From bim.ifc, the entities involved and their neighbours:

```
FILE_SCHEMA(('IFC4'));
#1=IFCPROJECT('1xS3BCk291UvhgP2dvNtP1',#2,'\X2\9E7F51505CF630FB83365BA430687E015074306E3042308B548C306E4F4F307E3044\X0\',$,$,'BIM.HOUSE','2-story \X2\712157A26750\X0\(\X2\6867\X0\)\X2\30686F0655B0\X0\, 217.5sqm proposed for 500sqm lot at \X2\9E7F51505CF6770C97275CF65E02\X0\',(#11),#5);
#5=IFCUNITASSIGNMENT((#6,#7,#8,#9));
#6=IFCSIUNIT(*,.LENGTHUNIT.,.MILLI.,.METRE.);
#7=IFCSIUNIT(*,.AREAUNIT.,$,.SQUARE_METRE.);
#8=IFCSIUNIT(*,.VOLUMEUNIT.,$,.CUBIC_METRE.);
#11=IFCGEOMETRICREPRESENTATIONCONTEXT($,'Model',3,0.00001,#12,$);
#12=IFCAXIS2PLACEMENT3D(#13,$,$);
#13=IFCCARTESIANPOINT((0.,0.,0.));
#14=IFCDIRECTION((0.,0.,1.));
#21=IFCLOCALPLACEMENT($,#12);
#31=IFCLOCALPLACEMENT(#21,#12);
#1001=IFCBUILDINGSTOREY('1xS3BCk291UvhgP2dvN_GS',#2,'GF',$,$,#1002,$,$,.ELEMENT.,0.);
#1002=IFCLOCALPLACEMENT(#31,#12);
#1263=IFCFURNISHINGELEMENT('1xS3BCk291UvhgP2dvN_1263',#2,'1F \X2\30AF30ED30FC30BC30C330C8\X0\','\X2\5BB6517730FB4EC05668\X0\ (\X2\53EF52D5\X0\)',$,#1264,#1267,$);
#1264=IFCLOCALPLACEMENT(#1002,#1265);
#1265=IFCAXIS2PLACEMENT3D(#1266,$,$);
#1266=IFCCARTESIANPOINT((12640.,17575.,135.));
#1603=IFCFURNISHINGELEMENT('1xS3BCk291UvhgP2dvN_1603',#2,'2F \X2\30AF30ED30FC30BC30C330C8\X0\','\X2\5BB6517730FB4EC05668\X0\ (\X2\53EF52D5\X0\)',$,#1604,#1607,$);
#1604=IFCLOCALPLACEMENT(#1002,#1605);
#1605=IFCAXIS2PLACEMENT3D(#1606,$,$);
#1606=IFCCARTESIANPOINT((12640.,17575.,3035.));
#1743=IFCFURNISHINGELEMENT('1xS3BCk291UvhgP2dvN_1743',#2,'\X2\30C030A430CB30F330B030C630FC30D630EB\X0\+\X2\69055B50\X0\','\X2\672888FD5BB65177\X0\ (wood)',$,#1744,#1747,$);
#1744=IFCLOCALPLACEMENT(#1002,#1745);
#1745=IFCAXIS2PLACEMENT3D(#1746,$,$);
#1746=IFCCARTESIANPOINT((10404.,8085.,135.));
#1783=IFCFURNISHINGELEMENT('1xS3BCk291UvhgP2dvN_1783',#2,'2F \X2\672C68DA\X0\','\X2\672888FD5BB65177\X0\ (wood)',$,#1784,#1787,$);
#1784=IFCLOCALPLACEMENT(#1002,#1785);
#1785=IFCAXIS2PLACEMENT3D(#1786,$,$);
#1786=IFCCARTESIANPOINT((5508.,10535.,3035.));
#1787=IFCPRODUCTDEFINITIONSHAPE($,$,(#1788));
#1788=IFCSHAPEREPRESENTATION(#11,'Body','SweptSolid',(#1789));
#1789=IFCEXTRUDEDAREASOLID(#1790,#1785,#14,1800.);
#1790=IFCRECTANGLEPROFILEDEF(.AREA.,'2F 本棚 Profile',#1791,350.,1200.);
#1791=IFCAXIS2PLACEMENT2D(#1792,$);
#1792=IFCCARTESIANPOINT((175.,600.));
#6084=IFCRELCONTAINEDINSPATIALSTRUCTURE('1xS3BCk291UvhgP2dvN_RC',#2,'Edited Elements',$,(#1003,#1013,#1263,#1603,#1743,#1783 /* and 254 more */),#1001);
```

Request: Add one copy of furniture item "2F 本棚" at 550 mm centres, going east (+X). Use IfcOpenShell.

```python
import numpy as np
import ifcopenshell
import ifcopenshell.api.geometry
import ifcopenshell.api.root
import ifcopenshell.util.element
import ifcopenshell.util.placement

model = ifcopenshell.open("bim.ifc")


def reuse_history(source, copy):
    """copy_class also copies each property set's owner history, people and application; keep the originals."""
    for rel in copy.IsDefinedBy:
        if rel.is_a("IfcRelDefinesByProperties") and (history := rel.RelatingPropertyDefinition.OwnerHistory):
            rel.RelatingPropertyDefinition.OwnerHistory = source.OwnerHistory
            ifcopenshell.util.element.remove_deep2(model, history)


source = model.by_id(1783)
base = ifcopenshell.util.placement.get_local_placement(source.ObjectPlacement)
step = np.array([1.0, 0.0, 0.0]) * 550.0

for i in range(1, 2):
    copy = ifcopenshell.api.root.copy_class(model, product=source)
    copy.Representation = ifcopenshell.util.element.copy_deep(
        model, source.Representation, exclude=["IfcGeometricRepresentationContext", "IfcRepresentationMap"]
    )
    reuse_history(source, copy)
    matrix = base.copy()
    matrix[:3, 3] += i * step
    print("added at", matrix[:3, 3].round(3) + 0.0)
    ifcopenshell.api.geometry.edit_object_placement(model, product=copy, matrix=matrix, is_si=False)

model.write("bim_updated.ifc")
```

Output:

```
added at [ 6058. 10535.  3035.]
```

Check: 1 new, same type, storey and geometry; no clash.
